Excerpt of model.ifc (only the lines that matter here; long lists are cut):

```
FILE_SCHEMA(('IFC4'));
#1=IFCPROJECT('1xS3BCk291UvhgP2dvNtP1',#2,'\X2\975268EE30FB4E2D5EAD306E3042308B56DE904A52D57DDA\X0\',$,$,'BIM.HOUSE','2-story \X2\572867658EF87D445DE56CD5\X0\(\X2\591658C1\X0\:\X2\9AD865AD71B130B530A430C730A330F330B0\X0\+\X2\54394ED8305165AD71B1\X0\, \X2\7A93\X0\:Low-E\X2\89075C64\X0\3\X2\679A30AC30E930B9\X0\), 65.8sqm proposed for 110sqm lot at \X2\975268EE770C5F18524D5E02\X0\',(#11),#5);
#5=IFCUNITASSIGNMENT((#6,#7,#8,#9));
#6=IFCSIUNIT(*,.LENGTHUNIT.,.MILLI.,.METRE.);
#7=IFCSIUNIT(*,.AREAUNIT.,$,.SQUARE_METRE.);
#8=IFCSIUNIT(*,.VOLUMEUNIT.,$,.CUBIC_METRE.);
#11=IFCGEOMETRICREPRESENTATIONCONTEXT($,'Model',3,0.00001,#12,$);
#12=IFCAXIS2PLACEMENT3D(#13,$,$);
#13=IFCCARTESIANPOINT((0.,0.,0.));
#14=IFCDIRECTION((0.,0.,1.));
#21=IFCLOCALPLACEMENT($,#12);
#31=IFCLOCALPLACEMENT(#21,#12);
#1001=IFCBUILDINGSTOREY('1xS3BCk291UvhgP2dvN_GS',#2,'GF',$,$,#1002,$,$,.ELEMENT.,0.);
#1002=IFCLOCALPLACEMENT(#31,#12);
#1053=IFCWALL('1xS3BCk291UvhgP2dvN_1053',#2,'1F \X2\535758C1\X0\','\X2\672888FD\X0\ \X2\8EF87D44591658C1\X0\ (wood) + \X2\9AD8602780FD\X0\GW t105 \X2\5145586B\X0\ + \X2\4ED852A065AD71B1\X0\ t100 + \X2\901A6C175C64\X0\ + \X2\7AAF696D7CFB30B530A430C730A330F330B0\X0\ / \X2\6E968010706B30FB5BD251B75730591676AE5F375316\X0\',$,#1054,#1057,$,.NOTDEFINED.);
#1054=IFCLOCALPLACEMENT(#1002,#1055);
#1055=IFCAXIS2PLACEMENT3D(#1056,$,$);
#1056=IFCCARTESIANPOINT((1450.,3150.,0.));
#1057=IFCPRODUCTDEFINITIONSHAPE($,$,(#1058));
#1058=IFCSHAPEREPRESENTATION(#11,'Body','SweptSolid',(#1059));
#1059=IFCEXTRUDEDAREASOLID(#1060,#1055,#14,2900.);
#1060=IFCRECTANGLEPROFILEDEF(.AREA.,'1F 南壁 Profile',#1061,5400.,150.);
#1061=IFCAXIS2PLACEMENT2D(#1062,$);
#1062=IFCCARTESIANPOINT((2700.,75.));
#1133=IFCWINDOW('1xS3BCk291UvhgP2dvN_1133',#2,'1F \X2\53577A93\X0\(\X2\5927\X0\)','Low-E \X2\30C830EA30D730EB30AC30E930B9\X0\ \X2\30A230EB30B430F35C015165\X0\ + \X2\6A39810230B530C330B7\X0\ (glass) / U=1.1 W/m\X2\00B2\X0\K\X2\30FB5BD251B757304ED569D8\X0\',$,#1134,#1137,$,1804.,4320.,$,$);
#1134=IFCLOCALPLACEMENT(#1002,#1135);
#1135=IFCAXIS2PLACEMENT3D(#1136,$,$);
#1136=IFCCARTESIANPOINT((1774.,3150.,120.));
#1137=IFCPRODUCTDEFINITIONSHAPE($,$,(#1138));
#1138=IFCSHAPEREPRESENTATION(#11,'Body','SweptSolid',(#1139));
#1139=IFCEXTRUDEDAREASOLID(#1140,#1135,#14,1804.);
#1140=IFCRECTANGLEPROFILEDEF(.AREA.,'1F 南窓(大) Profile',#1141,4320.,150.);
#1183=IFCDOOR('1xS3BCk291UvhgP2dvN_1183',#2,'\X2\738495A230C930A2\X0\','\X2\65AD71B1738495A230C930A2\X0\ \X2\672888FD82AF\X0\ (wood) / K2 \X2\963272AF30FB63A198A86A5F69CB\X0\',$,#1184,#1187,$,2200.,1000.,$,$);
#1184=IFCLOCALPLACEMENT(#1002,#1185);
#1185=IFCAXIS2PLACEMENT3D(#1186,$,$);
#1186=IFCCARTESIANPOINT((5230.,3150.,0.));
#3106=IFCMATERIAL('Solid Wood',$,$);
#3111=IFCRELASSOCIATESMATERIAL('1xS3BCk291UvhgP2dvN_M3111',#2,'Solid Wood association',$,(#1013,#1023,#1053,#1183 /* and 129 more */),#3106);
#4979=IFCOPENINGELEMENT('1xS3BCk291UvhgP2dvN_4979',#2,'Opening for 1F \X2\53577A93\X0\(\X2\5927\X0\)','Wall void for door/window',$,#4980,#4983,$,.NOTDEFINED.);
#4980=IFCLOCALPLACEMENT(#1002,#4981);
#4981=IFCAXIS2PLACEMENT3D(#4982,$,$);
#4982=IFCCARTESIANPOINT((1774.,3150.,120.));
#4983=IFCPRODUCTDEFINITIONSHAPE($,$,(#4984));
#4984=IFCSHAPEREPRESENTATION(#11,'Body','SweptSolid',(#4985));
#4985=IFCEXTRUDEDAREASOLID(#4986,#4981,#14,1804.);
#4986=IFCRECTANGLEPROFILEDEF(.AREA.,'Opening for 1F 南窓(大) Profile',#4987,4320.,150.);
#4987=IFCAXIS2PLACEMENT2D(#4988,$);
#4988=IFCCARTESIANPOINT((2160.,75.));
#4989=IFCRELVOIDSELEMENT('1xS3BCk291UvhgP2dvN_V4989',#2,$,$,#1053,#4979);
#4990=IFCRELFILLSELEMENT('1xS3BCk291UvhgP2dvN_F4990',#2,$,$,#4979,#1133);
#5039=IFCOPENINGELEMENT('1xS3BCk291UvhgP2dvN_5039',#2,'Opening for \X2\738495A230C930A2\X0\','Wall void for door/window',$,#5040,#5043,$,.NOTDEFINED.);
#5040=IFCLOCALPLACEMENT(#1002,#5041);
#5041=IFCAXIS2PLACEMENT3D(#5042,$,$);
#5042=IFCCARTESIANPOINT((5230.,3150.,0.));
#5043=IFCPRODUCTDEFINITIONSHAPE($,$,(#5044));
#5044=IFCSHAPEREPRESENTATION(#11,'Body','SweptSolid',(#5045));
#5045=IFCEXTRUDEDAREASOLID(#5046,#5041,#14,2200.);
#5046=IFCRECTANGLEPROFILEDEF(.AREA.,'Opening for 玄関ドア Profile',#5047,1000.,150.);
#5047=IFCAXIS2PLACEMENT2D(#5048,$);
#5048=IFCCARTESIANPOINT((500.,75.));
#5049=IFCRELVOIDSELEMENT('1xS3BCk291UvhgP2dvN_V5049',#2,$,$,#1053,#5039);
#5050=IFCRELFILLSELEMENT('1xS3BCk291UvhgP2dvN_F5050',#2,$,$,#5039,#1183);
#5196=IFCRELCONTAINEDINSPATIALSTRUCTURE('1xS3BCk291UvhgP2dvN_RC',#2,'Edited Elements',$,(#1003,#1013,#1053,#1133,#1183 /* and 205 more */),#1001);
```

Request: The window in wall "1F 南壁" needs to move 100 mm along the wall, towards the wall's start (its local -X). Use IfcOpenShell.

```python
import ifcopenshell
import ifcopenshell.api.geometry
import ifcopenshell.util.placement
import ifcopenshell.util.unit

model = ifcopenshell.open("model.ifc")
unit_scale = ifcopenshell.util.unit.calculate_unit_scale(model)

window = model.by_guid("1xS3BCk291UvhgP2dvN_1133")
opening = window.FillsVoids[0].RelatingOpeningElement
wall = opening.VoidsElements[0].RelatingBuildingElement

wall_matrix = ifcopenshell.util.placement.get_local_placement(wall.ObjectPlacement)
shift = wall_matrix[:3, 0] * -0.1 / unit_scale
before = ifcopenshell.util.placement.get_local_placement(window.ObjectPlacement)[:3, 3].copy()

# The window is not placed relative to its opening, so move both.
for product in (opening, window):
    matrix = ifcopenshell.util.placement.get_local_placement(product.ObjectPlacement)
    matrix[:3, 3] += shift
    ifcopenshell.api.geometry.edit_object_placement(model, product=product, matrix=matrix, is_si=False)

after = ifcopenshell.util.placement.get_local_placement(window.ObjectPlacement)[:3, 3]
print("window moved by", (after - before).round(3) + 0.0)

model.write("model-out.ifc")
```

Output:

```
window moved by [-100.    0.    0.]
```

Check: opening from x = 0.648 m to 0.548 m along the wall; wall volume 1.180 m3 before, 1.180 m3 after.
